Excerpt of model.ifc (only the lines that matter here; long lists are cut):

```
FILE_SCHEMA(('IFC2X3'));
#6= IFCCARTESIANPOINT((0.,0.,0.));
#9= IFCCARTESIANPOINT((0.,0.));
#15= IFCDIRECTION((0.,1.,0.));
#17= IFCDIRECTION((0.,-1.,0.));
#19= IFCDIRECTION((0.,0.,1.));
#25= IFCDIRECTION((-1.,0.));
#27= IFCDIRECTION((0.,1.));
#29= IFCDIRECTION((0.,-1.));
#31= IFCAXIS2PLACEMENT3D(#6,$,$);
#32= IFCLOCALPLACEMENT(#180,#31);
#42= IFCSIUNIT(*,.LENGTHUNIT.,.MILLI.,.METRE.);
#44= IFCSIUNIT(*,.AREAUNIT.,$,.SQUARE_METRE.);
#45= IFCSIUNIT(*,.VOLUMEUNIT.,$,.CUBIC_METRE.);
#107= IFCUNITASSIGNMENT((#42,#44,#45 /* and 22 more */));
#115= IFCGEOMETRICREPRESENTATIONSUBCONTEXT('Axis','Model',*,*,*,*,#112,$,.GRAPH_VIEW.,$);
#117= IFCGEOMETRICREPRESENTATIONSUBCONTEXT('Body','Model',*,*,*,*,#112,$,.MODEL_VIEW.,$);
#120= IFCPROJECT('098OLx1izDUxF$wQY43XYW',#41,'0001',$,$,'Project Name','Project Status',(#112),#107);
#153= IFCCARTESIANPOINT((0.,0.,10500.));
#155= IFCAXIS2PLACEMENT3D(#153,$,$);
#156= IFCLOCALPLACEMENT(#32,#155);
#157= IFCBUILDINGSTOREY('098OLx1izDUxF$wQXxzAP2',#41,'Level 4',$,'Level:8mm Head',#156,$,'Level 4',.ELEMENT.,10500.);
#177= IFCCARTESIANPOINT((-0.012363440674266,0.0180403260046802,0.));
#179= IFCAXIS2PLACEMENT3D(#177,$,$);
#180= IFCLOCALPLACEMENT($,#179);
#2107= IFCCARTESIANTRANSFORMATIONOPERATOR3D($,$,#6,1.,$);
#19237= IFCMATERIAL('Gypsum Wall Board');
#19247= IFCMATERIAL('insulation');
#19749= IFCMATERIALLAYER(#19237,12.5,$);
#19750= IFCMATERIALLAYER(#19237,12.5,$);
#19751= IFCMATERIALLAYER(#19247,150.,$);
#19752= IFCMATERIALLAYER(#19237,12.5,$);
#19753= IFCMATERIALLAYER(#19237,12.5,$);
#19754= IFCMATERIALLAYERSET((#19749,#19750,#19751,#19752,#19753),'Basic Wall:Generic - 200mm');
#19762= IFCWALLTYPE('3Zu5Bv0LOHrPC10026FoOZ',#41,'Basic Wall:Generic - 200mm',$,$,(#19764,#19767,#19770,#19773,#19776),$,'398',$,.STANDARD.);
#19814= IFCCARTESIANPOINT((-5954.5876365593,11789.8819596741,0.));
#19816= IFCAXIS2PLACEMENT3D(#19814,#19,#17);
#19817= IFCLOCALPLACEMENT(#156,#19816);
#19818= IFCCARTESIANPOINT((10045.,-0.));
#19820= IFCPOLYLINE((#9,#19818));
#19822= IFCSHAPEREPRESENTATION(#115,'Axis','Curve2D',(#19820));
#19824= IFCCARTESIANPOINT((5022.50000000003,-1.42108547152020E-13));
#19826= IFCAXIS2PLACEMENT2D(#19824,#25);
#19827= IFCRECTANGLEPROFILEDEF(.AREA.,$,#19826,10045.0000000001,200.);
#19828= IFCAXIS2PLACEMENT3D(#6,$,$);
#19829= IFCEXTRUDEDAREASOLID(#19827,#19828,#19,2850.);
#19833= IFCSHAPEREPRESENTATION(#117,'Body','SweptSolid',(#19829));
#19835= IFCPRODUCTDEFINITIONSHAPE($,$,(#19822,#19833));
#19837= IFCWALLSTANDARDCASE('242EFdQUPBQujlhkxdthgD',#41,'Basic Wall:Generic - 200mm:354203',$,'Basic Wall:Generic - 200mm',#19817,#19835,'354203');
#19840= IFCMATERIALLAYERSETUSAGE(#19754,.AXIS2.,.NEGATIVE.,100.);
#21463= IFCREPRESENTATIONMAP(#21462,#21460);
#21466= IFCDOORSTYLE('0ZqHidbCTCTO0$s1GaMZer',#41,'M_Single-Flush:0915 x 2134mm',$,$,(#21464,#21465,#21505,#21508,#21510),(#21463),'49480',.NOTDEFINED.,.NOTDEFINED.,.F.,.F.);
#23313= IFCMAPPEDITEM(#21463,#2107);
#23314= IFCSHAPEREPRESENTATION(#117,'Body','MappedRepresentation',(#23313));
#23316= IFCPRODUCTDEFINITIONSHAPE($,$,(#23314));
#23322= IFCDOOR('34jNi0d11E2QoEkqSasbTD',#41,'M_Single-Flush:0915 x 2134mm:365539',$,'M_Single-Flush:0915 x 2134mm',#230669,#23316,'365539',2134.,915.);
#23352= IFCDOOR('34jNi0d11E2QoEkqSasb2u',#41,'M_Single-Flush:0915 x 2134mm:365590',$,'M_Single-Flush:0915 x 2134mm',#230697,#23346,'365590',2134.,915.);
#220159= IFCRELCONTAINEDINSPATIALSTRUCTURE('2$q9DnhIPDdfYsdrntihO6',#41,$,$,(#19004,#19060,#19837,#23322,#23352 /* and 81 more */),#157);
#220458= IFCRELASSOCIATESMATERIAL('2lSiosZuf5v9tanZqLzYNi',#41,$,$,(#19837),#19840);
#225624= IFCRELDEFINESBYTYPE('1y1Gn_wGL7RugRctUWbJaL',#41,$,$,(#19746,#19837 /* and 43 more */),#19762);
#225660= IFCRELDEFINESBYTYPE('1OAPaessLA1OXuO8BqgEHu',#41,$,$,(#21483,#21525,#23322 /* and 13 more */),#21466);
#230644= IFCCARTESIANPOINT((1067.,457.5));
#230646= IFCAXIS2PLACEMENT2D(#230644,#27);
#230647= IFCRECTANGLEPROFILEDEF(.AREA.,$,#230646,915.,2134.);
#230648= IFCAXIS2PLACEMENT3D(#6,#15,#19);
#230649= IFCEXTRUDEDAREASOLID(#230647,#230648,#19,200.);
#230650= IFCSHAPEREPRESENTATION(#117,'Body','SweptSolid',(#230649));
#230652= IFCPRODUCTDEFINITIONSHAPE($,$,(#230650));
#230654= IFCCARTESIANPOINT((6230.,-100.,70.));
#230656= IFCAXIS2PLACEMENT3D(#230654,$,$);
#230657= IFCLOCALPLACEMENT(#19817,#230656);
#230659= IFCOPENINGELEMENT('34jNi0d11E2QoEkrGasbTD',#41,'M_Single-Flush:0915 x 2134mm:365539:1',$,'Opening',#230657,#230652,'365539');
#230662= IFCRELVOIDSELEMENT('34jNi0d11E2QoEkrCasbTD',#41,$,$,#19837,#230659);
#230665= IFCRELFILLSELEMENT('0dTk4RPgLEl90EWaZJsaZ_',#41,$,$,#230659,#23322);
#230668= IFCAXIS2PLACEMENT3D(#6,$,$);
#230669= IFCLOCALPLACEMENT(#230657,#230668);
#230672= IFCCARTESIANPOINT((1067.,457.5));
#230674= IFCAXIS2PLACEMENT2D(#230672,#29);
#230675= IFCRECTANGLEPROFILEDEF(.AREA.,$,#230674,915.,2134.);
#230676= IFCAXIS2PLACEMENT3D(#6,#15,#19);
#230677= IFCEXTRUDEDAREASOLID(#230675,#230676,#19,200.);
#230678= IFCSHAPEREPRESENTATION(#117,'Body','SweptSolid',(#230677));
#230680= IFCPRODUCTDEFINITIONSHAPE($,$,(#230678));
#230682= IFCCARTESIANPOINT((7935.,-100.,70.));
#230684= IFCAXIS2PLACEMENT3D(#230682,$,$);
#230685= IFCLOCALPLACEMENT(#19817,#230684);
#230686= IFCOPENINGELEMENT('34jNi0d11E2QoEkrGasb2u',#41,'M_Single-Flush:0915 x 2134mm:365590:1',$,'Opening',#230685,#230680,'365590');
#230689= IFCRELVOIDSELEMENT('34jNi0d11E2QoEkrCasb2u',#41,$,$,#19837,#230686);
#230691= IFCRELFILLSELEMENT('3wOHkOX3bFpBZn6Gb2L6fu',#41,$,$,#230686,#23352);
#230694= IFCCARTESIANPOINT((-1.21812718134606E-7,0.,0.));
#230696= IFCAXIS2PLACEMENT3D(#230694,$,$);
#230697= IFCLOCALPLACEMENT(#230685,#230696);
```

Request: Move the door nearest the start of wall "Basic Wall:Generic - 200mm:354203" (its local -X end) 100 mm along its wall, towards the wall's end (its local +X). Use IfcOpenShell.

```python
import ifcopenshell
import ifcopenshell.api.geometry
import ifcopenshell.util.placement

model = ifcopenshell.open("model.ifc")

door = model.by_id(23322)
opening = door.FillsVoids[0].RelatingOpeningElement
wall = opening.VoidsElements[0].RelatingBuildingElement

wall_matrix = ifcopenshell.util.placement.get_local_placement(wall.ObjectPlacement)
shift = wall_matrix[:3, 0] * 100.0
before = ifcopenshell.util.placement.get_local_placement(door.ObjectPlacement)[:3, 3].copy()

# The door is placed relative to its opening, so it follows when the opening moves.
matrix = ifcopenshell.util.placement.get_local_placement(opening.ObjectPlacement)
matrix[:3, 3] += shift
ifcopenshell.api.geometry.edit_object_placement(
    model, product=opening, matrix=matrix, is_si=False, should_transform_children=True
)

after = ifcopenshell.util.placement.get_local_placement(door.ObjectPlacement)[:3, 3]
print("door moved by", (after - before).round(3) + 0.0)

model.write("model_edited.ifc")
```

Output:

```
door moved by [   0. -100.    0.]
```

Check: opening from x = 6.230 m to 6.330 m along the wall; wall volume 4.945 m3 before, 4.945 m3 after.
